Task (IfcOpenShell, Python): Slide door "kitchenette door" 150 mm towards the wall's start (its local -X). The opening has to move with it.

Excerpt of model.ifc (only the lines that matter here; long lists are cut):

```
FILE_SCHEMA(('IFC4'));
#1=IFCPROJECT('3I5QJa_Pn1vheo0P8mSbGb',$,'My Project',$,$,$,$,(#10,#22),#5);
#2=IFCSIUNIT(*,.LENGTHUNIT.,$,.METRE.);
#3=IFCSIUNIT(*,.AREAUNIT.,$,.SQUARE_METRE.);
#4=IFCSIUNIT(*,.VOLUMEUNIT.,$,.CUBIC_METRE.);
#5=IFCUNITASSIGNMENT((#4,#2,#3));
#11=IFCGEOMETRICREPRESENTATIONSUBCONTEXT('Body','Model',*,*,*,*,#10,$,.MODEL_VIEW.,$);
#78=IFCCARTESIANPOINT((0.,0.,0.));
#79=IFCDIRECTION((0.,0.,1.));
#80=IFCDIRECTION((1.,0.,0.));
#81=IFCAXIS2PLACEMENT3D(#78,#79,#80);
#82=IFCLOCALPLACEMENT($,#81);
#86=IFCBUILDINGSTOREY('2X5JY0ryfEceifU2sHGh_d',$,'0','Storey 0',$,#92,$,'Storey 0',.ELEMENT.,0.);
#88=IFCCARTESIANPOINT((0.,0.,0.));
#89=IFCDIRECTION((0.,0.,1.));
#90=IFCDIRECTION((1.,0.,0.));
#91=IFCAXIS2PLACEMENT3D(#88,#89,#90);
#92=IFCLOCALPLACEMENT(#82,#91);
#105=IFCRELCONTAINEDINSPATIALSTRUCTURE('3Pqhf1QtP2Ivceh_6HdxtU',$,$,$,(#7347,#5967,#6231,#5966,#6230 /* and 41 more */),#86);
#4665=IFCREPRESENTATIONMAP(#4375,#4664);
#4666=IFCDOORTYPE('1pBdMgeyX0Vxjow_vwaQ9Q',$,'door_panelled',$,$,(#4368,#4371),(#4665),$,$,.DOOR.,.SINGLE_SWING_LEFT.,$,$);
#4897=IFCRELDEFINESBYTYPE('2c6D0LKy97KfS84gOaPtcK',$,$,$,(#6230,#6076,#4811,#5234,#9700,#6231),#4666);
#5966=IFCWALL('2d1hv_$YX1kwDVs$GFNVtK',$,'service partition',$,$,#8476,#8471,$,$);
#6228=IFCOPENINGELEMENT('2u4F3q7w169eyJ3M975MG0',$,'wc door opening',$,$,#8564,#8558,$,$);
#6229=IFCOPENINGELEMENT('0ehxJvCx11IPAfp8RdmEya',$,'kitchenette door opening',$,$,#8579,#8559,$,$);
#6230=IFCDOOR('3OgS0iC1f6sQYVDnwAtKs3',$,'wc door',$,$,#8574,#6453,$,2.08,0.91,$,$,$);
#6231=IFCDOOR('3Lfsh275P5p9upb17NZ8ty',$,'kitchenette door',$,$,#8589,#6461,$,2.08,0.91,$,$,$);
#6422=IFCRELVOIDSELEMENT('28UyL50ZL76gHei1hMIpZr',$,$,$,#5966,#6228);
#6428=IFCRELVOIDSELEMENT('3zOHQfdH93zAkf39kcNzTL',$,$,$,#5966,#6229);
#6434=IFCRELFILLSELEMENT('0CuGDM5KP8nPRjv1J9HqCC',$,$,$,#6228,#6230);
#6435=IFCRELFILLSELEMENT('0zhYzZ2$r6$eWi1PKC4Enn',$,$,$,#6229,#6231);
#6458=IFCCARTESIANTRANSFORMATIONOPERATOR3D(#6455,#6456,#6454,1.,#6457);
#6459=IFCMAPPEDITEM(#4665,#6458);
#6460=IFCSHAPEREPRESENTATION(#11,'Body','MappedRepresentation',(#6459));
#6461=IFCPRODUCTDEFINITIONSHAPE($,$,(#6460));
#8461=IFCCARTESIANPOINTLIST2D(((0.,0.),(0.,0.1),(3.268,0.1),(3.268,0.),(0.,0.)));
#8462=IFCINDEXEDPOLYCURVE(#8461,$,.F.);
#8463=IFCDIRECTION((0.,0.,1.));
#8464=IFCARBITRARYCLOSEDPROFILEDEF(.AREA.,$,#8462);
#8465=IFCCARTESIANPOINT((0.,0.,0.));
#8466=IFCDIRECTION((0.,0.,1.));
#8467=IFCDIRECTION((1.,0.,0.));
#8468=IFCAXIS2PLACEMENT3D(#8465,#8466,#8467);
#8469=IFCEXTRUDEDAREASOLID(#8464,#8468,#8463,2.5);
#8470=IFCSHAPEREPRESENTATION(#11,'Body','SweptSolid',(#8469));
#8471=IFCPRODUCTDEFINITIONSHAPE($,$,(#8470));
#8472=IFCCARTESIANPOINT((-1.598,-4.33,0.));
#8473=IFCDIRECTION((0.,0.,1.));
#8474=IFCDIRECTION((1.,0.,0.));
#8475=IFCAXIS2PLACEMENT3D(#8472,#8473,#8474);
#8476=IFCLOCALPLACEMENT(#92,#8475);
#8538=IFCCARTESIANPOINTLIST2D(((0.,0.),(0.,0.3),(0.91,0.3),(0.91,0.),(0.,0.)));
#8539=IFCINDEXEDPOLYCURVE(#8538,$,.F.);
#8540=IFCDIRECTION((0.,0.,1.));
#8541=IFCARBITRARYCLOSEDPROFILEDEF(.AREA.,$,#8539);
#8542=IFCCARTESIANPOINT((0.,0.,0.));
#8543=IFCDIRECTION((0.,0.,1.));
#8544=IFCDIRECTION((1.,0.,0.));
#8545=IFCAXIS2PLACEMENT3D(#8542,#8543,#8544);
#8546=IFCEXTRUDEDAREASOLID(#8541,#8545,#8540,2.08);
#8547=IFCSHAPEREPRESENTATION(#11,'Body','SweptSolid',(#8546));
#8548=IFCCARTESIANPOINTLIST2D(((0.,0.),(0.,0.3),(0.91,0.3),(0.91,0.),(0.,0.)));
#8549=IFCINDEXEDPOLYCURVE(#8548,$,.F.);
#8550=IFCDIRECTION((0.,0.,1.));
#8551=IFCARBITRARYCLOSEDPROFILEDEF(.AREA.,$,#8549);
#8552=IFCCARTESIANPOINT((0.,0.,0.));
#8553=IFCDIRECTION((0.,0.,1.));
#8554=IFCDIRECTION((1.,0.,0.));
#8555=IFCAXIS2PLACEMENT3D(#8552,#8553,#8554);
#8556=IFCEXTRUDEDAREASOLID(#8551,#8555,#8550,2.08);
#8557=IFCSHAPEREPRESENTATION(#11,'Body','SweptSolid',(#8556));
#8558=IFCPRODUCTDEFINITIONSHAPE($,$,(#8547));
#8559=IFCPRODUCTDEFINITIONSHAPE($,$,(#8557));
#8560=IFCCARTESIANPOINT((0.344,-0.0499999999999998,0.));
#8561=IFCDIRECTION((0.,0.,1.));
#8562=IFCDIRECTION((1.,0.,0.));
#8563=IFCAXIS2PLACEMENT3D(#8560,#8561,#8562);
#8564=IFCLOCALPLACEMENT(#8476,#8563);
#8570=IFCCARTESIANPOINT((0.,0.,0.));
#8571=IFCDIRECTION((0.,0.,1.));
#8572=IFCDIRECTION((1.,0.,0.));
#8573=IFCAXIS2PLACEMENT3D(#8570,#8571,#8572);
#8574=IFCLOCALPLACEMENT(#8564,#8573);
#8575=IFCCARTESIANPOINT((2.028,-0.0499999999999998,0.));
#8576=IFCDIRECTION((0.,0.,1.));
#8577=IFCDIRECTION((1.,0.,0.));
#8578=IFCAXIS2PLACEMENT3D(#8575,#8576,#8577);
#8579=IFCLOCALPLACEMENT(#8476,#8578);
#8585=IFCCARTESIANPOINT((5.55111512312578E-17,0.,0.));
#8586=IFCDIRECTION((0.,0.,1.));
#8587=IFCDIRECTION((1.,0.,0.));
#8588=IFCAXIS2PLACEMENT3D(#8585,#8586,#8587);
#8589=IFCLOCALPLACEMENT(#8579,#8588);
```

```python
import ifcopenshell
import ifcopenshell.api.geometry
import ifcopenshell.util.placement
import ifcopenshell.util.unit

model = ifcopenshell.open("model.ifc")
unit_scale = ifcopenshell.util.unit.calculate_unit_scale(model)

door = model.by_id(6231)
opening = door.FillsVoids[0].RelatingOpeningElement
wall = opening.VoidsElements[0].RelatingBuildingElement

wall_matrix = ifcopenshell.util.placement.get_local_placement(wall.ObjectPlacement)
shift = wall_matrix[:3, 0] * -0.15 / unit_scale
before = ifcopenshell.util.placement.get_local_placement(door.ObjectPlacement)[:3, 3].copy()

# The door is placed relative to its opening, so it follows when the opening moves.
matrix = ifcopenshell.util.placement.get_local_placement(opening.ObjectPlacement)
matrix[:3, 3] += shift
ifcopenshell.api.geometry.edit_object_placement(
    model, product=opening, matrix=matrix, is_si=False, should_transform_children=True
)

after = ifcopenshell.util.placement.get_local_placement(door.ObjectPlacement)[:3, 3]
print("door moved by", (after - before).round(3) + 0.0)

model.write("model-out.ifc")
```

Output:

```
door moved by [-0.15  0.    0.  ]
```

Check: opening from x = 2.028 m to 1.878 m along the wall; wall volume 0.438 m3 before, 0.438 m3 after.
